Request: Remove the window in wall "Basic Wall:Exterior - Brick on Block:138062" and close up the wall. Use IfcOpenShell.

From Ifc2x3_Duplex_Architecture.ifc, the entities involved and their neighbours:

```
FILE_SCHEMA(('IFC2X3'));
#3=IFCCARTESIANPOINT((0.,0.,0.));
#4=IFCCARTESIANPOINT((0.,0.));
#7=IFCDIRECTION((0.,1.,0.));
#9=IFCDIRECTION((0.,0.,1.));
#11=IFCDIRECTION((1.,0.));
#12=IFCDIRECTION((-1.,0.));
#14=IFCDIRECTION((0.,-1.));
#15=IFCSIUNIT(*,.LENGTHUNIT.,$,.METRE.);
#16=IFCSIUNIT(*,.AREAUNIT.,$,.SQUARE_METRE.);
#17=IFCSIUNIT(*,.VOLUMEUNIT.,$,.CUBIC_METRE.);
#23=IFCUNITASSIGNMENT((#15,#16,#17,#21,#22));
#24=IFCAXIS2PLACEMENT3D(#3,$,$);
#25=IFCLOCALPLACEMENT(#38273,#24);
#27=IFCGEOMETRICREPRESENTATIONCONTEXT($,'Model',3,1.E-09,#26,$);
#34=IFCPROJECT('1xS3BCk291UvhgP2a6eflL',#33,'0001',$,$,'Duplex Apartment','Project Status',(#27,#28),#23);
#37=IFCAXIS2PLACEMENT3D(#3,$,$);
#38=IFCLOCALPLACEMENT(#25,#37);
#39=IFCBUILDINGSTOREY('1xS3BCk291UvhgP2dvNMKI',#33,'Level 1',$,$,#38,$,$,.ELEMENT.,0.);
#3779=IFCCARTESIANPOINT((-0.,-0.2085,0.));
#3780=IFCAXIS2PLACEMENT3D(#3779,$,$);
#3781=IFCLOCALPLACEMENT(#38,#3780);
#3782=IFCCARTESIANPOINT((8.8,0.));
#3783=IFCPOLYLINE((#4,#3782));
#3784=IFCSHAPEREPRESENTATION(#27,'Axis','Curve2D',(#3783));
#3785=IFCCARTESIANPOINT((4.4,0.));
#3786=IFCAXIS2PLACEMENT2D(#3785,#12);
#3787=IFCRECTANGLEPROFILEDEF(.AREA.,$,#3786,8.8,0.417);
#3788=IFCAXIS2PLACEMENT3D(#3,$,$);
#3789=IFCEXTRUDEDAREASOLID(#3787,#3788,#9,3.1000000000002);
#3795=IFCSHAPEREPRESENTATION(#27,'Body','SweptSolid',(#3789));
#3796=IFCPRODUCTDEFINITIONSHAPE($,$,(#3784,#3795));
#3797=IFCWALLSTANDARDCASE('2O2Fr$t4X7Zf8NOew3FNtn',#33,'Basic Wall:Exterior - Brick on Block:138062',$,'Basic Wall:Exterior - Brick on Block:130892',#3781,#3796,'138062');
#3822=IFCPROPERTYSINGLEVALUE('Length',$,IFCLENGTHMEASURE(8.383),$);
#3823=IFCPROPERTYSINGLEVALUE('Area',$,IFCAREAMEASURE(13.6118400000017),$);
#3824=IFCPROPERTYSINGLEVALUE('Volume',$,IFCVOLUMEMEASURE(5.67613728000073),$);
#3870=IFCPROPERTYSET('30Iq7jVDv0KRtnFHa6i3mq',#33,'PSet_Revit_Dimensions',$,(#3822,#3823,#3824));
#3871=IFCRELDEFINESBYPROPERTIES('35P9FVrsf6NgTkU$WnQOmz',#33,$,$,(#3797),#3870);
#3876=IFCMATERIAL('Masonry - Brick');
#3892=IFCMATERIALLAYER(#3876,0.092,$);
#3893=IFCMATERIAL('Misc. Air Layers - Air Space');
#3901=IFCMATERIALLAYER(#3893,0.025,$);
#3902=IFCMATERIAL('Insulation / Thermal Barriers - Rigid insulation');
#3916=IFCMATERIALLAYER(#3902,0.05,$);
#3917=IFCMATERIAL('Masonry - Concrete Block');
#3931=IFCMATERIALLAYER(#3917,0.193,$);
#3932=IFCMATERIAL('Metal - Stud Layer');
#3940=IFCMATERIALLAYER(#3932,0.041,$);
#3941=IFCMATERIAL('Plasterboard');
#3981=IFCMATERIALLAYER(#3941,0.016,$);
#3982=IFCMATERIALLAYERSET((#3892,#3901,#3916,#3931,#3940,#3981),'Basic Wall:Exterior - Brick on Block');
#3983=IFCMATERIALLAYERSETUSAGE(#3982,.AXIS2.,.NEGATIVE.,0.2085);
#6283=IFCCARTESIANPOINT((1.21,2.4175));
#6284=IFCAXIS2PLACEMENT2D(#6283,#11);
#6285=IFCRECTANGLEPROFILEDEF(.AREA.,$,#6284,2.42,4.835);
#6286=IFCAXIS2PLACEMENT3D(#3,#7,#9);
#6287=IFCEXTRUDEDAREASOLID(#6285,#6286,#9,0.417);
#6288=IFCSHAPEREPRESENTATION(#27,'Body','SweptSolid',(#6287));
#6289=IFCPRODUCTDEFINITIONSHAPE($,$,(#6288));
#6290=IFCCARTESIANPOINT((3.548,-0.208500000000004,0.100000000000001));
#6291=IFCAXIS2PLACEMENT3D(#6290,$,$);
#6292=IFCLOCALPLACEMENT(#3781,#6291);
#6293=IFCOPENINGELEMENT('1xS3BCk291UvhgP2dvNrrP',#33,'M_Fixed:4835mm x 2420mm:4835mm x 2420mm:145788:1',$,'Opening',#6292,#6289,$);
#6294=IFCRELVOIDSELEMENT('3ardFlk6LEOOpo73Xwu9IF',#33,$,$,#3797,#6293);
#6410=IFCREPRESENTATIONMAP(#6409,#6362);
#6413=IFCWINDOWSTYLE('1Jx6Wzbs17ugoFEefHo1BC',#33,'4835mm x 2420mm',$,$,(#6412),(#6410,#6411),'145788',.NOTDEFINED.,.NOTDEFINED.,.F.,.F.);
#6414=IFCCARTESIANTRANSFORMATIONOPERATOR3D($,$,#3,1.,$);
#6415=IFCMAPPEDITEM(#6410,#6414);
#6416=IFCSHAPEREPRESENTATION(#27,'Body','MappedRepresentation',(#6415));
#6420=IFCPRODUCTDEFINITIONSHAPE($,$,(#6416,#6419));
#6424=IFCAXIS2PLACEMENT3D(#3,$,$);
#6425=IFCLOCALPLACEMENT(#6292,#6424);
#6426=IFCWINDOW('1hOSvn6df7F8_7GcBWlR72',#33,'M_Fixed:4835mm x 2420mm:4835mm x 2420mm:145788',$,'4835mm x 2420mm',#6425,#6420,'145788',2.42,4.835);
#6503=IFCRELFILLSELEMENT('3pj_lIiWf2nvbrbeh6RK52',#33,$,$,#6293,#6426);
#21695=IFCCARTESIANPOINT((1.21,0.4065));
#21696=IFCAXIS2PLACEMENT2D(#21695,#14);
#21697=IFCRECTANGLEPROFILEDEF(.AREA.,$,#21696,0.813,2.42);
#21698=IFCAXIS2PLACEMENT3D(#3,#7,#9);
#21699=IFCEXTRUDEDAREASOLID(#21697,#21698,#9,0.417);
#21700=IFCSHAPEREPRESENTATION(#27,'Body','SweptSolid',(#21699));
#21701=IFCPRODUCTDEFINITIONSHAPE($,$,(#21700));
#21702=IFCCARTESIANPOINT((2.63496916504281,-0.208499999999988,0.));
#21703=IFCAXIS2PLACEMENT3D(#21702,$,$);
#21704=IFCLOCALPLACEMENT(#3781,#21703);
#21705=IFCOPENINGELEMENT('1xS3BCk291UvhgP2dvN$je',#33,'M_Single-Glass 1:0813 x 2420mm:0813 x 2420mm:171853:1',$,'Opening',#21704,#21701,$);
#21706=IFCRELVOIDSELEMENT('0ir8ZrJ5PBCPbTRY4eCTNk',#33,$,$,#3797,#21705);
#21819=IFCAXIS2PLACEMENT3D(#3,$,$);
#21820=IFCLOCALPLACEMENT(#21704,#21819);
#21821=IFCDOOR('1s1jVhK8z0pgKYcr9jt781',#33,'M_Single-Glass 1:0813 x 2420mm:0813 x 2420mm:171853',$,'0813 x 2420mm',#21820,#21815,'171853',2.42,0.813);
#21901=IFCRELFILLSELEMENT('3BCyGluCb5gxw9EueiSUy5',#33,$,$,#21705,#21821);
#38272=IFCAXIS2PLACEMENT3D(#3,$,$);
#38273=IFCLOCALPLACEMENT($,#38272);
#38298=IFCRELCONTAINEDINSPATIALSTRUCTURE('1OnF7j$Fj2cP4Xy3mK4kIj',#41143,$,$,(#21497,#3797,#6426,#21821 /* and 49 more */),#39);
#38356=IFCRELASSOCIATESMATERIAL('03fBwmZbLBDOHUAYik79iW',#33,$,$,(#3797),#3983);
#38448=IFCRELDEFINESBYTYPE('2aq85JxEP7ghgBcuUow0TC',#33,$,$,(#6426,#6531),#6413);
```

```python
import ifcopenshell
import ifcopenshell.api.feature
import ifcopenshell.api.pset
import ifcopenshell.api.root
import ifcopenshell.geom
import ifcopenshell.util.element
import ifcopenshell.util.shape
import ifcopenshell.util.unit

model = ifcopenshell.open("Ifc2x3_Duplex_Architecture.ifc")
area_scale = ifcopenshell.util.unit.calculate_unit_scale(model, "AREAUNIT")
volume_scale = ifcopenshell.util.unit.calculate_unit_scale(model, "VOLUMEUNIT")
settings = ifcopenshell.geom.settings()


def volume(element):
    """Net volume in cubic metres, openings subtracted."""
    shape = ifcopenshell.geom.create_shape(settings, element)
    return ifcopenshell.util.shape.get_volume(shape.geometry)


window = model.by_guid("1hOSvn6df7F8_7GcBWlR72")
opening = window.FillsVoids[0].RelatingOpeningElement
wall = opening.VoidsElements[0].RelatingBuildingElement
before = volume(wall)

ifcopenshell.api.root.remove_product(model, product=window)
ifcopenshell.api.feature.remove_feature(model, feature=opening)

after = volume(wall)
thickness = 0.417  # wall thickness in metres

# Update the wall's stored quantities.
pset = model.by_id(ifcopenshell.util.element.get_pset(wall, "PSet_Revit_Dimensions", should_inherit=False)["id"])
ifcopenshell.api.pset.edit_pset(model, pset=pset, properties={
    "Area": model.create_entity("IfcAreaMeasure", after / thickness / area_scale),
    "Volume": model.create_entity("IfcVolumeMeasure", after / volume_scale),
})

print(f"wall volume {before:.3f} -> {after:.3f} m3")

model.write("Ifc2x3_Duplex_Architecture_edited.ifc")
```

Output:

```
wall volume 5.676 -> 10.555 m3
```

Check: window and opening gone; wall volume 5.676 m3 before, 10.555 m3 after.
